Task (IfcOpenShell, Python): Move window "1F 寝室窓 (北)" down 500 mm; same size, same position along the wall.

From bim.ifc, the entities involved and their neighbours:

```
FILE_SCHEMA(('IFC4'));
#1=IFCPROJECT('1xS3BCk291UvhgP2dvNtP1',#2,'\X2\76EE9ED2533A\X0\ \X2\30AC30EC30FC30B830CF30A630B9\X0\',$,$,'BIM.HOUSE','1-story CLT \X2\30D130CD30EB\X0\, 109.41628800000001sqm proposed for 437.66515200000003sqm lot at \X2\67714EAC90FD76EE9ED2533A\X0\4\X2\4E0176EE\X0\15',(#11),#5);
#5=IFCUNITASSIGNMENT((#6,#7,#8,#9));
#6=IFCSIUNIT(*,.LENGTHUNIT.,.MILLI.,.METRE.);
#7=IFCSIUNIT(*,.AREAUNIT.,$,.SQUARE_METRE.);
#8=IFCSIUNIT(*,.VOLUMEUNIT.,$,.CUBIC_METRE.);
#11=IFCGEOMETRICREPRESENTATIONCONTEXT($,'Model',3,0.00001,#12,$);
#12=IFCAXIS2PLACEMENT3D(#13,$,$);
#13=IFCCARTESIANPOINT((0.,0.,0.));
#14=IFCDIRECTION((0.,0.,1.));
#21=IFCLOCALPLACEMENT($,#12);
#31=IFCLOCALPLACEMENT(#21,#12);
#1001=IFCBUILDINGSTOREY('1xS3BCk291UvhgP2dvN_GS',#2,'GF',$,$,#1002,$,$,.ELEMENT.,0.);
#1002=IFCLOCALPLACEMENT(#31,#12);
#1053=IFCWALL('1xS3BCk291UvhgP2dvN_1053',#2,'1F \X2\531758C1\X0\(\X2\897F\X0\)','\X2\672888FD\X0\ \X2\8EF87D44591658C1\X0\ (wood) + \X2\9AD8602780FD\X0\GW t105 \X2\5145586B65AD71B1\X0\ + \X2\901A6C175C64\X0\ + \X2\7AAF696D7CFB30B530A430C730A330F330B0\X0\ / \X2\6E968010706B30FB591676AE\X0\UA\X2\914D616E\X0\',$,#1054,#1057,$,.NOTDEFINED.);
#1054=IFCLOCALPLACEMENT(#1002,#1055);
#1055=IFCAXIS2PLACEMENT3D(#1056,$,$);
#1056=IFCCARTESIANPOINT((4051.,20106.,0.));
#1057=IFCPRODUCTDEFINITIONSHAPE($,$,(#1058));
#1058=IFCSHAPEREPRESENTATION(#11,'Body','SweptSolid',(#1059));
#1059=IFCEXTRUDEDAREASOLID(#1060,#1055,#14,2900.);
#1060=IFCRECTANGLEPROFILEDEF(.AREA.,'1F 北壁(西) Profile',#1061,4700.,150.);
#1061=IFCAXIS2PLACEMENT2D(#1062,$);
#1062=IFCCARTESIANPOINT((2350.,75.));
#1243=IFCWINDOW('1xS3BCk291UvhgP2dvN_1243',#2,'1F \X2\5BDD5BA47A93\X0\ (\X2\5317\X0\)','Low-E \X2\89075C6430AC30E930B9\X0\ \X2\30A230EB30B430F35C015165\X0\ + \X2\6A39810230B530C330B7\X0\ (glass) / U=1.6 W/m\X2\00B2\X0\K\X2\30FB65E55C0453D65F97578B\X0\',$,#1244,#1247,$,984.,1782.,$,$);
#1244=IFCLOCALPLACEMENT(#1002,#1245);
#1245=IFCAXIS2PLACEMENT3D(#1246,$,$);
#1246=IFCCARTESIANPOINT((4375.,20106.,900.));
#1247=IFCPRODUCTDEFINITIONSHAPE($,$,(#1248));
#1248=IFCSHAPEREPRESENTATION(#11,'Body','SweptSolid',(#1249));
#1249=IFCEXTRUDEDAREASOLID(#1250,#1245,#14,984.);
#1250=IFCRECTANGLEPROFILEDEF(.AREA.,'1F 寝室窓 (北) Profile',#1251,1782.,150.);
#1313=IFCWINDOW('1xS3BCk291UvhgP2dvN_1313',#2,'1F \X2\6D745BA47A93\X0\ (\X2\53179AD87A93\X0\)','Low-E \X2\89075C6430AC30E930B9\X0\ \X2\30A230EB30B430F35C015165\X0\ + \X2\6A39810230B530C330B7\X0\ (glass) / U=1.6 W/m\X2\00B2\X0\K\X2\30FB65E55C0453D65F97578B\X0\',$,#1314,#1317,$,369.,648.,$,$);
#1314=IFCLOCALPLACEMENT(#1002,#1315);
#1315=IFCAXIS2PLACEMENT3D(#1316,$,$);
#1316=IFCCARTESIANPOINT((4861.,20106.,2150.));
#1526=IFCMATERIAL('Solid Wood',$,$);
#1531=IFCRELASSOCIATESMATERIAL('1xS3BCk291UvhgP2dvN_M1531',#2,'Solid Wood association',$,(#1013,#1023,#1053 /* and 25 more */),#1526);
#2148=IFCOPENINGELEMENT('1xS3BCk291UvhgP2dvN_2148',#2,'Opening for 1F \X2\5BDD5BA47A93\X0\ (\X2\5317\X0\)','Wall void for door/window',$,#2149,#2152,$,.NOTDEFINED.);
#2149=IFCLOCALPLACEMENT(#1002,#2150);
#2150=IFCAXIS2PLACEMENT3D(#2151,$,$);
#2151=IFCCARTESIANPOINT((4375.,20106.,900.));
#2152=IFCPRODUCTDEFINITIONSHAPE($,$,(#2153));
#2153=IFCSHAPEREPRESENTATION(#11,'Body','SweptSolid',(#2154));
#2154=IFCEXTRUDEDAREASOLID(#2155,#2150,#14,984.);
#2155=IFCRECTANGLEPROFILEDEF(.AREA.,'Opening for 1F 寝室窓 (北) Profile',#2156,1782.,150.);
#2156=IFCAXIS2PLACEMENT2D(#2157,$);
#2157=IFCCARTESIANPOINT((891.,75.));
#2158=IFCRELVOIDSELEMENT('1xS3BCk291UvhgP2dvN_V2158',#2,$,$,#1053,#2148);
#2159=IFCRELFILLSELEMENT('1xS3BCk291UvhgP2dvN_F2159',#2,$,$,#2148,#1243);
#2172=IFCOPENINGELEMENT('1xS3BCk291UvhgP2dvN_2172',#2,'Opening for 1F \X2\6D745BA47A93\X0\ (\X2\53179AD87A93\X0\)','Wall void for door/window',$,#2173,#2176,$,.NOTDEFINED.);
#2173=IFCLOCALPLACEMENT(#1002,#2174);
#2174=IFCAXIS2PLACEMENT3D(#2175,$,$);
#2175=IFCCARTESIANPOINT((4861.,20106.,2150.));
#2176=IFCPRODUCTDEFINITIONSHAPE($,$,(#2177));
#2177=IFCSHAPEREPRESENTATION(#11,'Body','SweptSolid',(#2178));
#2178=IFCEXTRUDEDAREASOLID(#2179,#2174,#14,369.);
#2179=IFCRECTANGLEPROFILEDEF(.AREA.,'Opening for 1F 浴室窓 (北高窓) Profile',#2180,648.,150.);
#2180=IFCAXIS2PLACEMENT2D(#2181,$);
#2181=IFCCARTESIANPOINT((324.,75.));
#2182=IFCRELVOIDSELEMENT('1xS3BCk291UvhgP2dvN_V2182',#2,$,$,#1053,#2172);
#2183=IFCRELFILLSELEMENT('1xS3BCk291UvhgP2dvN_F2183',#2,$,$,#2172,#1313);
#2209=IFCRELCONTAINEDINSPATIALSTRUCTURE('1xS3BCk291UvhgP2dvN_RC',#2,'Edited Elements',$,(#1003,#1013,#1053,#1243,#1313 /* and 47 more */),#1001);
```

```python
import numpy as np
import ifcopenshell
import ifcopenshell.api.geometry
import ifcopenshell.util.placement
import ifcopenshell.util.unit

model = ifcopenshell.open("bim.ifc")
unit_scale = ifcopenshell.util.unit.calculate_unit_scale(model)

window = model.by_id(1243)
opening = window.FillsVoids[0].RelatingOpeningElement
dz = -500.0

shift = np.array([0.0, 0.0, dz])
# The window is not placed relative to its opening, so move both.
for product in (opening, window):
    matrix = ifcopenshell.util.placement.get_local_placement(product.ObjectPlacement)
    matrix[:3, 3] += shift
    ifcopenshell.api.geometry.edit_object_placement(model, product=product, matrix=matrix, is_si=False)

print(f"moved by {dz * unit_scale:+.3f} m")

model.write("bim_edited.ifc")
```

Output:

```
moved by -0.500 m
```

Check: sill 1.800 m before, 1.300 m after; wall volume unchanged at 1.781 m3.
